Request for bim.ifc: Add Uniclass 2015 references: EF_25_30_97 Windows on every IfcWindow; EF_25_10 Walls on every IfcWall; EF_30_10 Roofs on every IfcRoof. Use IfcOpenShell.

First a look at what the model holds.

```python
import ifcopenshell

model = ifcopenshell.open("bim.ifc")
print(model.schema)
print("classifications:", [c.Name for c in model.by_type("IfcClassification")])
for ifc_class in ("IfcDoor", "IfcRoof", "IfcStair", "IfcWall", "IfcWindow"):
    print(ifc_class, len(model.by_type(ifc_class)))
```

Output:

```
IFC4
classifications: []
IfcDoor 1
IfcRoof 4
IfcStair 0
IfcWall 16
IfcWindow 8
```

```python
import ifcopenshell
import ifcopenshell.api.classification

model = ifcopenshell.open("bim.ifc")

system = ifcopenshell.api.classification.add_classification(model, classification="Uniclass 2015")

codes = {
    "IfcWindow": ("EF_25_30_97", "Windows"),
    "IfcWall": ("EF_25_10", "Walls"),
    "IfcRoof": ("EF_30_10", "Roofs"),
}
for ifc_class, (code, name) in codes.items():
    products = model.by_type(ifc_class)
    ifcopenshell.api.classification.add_reference(
        model, products=products, classification=system, identification=code, name=name
    )
    print(code, len(products))

model.write("bim_edited.ifc")
```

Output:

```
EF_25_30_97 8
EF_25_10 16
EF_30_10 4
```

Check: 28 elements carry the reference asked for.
